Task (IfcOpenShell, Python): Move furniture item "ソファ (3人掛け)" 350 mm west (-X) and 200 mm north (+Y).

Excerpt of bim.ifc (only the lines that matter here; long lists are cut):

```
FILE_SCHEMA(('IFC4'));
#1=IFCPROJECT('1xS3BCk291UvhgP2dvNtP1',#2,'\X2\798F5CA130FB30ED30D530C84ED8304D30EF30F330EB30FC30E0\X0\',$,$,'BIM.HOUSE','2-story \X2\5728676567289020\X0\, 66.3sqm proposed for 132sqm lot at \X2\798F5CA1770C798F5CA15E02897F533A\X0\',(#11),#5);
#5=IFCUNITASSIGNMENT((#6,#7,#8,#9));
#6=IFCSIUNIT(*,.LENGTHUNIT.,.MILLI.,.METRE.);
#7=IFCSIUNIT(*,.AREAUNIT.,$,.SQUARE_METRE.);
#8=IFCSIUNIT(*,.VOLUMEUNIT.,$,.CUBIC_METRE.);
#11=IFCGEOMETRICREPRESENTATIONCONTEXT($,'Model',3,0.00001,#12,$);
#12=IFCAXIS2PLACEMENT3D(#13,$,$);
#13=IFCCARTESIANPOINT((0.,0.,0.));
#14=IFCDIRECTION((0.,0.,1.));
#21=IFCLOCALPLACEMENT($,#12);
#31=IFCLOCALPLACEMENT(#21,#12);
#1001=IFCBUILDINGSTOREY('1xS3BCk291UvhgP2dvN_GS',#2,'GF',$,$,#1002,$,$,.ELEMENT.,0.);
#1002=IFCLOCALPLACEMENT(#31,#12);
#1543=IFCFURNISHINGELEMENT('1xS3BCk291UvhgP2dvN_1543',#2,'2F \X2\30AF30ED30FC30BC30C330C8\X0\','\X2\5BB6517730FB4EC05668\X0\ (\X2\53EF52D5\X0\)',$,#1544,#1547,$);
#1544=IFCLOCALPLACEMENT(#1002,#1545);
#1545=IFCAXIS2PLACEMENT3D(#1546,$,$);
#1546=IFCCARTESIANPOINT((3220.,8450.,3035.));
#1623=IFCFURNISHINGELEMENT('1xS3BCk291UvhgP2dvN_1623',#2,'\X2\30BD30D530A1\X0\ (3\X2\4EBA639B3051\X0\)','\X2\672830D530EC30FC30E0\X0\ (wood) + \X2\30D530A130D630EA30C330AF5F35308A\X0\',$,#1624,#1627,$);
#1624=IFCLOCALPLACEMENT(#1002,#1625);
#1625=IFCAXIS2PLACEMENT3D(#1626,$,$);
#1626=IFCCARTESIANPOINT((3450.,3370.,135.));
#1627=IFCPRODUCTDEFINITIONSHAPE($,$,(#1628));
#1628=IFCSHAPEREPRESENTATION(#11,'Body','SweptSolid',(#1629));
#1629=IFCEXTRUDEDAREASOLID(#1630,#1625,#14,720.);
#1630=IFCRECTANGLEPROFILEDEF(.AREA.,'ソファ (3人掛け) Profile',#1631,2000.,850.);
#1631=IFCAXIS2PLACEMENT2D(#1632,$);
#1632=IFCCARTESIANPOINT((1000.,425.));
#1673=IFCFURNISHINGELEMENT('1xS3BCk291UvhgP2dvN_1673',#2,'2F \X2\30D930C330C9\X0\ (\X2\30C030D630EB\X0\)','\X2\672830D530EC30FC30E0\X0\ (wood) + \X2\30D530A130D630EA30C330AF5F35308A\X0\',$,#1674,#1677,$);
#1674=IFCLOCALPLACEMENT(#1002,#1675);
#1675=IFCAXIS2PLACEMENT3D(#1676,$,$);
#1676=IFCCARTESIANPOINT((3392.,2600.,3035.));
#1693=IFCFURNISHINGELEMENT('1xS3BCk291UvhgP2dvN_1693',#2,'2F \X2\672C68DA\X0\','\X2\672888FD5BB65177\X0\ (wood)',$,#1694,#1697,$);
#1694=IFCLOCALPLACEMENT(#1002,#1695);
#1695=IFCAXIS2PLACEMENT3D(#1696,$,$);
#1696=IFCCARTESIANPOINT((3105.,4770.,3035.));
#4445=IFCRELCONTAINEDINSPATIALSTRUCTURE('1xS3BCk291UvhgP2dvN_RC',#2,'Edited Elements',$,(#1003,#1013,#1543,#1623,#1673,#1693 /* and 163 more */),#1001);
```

```python
import ifcopenshell
import ifcopenshell.api.geometry
import ifcopenshell.util.placement

model = ifcopenshell.open("bim.ifc")

item = model.by_guid("1xS3BCk291UvhgP2dvN_1623")
matrix = ifcopenshell.util.placement.get_local_placement(item.ObjectPlacement)
matrix[0, 3] -= 350.0
matrix[1, 3] += 200.0
ifcopenshell.api.geometry.edit_object_placement(model, product=item, matrix=matrix, is_si=False)

print(ifcopenshell.util.placement.get_local_placement(item.ObjectPlacement).round(3) + 0.0)

model.write("bim_rev.ifc")
```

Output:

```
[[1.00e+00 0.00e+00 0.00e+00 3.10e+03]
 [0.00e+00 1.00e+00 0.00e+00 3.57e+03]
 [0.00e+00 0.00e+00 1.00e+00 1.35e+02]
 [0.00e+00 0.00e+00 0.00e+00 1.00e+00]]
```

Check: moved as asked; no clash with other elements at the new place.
